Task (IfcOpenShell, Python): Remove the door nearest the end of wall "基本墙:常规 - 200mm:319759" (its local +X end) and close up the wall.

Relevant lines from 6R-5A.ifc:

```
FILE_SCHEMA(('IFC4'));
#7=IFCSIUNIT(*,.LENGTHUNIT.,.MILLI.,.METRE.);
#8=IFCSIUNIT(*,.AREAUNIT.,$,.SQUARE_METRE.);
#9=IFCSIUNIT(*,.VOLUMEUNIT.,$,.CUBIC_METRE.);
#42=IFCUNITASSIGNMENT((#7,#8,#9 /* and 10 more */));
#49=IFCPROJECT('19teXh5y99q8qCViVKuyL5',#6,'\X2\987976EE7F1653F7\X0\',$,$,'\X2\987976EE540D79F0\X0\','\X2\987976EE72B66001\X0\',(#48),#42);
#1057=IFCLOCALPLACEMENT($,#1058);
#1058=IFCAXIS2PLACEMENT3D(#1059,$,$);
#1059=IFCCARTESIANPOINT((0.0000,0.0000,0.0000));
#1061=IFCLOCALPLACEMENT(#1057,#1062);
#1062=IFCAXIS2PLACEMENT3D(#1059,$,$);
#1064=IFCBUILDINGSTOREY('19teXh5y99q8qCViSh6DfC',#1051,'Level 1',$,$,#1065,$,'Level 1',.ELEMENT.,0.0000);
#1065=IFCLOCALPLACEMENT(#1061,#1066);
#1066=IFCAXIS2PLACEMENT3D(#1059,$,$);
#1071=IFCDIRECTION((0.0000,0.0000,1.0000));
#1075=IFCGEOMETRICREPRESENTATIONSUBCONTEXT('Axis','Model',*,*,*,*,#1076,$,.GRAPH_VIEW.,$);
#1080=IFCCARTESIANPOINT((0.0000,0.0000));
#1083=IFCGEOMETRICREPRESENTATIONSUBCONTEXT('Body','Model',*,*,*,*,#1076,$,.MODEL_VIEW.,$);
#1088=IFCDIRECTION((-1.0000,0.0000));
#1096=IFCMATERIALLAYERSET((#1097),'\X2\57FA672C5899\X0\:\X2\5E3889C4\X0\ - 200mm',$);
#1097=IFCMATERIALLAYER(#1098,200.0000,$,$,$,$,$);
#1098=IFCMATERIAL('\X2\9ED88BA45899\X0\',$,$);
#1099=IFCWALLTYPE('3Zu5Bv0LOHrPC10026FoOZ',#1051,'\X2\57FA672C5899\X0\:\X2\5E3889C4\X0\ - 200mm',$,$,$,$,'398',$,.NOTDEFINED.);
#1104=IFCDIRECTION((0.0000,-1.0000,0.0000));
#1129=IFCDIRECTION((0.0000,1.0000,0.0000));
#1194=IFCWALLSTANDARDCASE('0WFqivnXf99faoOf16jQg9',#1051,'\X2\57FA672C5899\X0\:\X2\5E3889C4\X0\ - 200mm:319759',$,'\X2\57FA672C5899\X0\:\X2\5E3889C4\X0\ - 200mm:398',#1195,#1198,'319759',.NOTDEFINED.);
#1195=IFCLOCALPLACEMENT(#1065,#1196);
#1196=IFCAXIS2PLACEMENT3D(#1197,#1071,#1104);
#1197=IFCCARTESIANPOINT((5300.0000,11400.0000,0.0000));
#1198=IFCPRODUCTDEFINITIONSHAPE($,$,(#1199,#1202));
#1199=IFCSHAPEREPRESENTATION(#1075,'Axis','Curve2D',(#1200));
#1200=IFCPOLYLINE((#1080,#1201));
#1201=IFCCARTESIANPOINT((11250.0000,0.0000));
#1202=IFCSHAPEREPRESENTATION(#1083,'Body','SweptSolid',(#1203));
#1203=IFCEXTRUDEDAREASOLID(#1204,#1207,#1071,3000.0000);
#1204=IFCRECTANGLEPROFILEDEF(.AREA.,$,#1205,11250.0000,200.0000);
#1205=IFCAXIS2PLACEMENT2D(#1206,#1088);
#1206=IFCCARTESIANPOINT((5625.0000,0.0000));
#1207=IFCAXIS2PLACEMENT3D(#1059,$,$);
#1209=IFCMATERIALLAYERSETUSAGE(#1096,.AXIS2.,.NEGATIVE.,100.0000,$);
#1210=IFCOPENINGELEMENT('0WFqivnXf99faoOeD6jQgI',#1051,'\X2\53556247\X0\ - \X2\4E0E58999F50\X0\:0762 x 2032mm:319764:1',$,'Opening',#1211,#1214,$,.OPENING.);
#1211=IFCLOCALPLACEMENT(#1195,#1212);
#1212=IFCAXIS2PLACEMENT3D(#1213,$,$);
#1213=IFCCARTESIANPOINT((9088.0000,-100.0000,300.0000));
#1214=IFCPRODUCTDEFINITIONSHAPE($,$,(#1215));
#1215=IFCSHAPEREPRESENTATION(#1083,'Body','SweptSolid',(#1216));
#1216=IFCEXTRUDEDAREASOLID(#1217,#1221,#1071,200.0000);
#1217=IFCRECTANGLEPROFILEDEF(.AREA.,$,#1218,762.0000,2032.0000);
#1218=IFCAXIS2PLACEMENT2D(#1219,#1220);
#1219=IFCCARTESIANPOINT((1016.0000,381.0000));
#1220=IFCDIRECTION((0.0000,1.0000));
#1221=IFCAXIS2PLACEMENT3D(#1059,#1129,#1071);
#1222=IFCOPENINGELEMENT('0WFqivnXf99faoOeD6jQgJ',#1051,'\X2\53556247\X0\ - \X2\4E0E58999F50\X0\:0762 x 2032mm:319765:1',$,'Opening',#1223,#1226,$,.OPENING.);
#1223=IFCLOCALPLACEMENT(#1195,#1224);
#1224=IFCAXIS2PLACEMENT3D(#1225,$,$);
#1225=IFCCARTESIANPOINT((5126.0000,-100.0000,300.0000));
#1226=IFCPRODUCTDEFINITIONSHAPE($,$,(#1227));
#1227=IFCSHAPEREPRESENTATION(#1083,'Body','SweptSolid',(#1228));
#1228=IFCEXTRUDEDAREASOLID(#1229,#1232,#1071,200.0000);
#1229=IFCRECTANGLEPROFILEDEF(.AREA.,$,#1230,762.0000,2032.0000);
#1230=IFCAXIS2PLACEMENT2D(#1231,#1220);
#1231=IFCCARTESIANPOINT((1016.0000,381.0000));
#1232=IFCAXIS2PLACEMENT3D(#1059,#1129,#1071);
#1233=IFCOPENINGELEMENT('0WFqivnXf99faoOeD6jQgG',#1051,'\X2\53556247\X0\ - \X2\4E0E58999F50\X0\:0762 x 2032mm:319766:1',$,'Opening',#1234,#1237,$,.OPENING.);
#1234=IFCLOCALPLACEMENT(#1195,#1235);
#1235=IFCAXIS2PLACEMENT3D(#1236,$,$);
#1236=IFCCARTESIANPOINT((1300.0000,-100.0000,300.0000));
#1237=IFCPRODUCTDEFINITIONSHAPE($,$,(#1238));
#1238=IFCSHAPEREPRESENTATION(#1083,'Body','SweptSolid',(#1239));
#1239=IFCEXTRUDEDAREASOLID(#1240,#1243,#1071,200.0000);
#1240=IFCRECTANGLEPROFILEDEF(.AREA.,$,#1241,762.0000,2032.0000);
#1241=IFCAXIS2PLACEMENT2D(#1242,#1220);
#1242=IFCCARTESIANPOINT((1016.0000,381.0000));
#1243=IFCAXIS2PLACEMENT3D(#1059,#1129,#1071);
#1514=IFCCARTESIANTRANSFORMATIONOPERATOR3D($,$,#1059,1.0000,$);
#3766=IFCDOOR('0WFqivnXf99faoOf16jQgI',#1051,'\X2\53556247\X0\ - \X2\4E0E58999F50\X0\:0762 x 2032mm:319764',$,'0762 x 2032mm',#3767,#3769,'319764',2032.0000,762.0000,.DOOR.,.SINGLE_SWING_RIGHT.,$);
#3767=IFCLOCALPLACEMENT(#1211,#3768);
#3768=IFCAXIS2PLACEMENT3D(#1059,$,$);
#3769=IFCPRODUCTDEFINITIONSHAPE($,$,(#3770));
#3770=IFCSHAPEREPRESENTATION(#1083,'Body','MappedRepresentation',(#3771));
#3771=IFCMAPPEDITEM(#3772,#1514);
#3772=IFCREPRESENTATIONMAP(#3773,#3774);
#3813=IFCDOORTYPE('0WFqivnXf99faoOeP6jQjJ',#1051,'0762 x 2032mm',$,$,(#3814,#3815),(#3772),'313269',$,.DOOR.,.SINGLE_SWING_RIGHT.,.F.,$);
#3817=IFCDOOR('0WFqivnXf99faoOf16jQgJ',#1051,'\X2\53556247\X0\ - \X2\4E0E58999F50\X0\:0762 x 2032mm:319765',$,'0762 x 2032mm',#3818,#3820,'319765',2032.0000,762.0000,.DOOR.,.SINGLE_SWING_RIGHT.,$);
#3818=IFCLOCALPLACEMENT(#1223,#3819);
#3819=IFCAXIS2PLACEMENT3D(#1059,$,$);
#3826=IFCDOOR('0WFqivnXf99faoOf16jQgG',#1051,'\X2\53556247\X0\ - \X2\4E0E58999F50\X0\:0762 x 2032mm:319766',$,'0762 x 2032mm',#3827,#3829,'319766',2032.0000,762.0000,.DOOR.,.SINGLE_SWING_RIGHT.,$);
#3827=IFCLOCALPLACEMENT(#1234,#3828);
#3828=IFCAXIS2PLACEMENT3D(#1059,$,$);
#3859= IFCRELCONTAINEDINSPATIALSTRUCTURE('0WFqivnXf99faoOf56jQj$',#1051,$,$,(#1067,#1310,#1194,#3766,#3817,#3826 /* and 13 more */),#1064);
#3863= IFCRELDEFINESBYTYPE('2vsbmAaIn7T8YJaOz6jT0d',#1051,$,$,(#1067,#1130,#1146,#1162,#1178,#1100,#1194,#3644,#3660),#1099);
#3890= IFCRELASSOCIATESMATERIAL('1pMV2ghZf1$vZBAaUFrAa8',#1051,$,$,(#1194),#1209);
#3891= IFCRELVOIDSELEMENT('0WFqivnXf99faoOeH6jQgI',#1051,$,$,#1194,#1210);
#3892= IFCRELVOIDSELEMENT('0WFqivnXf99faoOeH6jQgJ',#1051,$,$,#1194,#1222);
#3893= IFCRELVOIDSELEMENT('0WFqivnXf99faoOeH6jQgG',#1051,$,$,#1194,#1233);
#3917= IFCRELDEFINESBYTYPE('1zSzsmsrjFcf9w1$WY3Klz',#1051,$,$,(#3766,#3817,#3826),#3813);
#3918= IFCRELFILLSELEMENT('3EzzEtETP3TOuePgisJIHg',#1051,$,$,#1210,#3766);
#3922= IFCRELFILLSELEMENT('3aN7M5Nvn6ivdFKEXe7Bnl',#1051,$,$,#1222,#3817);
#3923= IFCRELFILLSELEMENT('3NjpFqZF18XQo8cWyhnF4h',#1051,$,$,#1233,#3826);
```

```python
import ifcopenshell
import ifcopenshell.api.feature
import ifcopenshell.api.root
import ifcopenshell.geom
import ifcopenshell.util.shape

model = ifcopenshell.open("6R-5A.ifc")
settings = ifcopenshell.geom.settings()


def volume(element):
    """Net volume in cubic metres, openings subtracted."""
    shape = ifcopenshell.geom.create_shape(settings, element)
    return ifcopenshell.util.shape.get_volume(shape.geometry)


door = model.by_id(3766)
opening = door.FillsVoids[0].RelatingOpeningElement
wall = opening.VoidsElements[0].RelatingBuildingElement
before = volume(wall)

ifcopenshell.api.root.remove_product(model, product=door)
ifcopenshell.api.feature.remove_feature(model, feature=opening)

after = volume(wall)

print(f"wall volume {before:.3f} -> {after:.3f} m3")

model.write("6R-5A_rev.ifc")
```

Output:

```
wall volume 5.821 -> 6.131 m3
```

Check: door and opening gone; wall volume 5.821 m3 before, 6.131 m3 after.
